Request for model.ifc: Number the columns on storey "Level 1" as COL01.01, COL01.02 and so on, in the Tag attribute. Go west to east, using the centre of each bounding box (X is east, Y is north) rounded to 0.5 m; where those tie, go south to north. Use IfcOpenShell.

First a look at what the model holds.

```python
import ifcopenshell
import ifcopenshell.util.element
import ifcopenshell.util.placement

model = ifcopenshell.open("model.ifc")
print(model.schema)
storey = next(s for s in model.by_type("IfcBuildingStorey") if s.Name == "Level 1")
columns = [e for e in ifcopenshell.util.element.get_decomposition(storey) if e.is_a("IfcColumn")]
for e in sorted(columns, key=lambda e: e.id()):
    origin = ifcopenshell.util.placement.get_local_placement(e.ObjectPlacement)[:3, 3]
    print(e.id(), e.Tag, e.Name, origin.round(2) + 0.0, sep=" | ")
```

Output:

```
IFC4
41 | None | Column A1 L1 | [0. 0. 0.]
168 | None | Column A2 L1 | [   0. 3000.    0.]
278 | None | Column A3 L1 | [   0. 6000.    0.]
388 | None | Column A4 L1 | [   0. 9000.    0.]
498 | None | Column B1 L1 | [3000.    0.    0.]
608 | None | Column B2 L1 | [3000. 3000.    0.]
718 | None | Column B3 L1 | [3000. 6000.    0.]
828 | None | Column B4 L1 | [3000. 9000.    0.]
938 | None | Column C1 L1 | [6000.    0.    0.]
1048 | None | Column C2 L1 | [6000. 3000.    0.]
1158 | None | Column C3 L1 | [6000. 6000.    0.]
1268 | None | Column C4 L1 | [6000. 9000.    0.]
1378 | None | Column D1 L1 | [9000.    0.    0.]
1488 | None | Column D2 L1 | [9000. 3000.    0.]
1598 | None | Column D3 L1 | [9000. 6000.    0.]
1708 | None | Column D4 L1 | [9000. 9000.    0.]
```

```python
import ifcopenshell
import ifcopenshell.geom
import ifcopenshell.util.element
import ifcopenshell.util.shape

model = ifcopenshell.open("model.ifc")
settings = ifcopenshell.geom.settings()
settings.set("use-world-coords", True)


def centre(element):
    shape = ifcopenshell.geom.create_shape(settings, element)
    return ifcopenshell.util.shape.get_bbox_centroid(shape.geometry)


storey = next(s for s in model.by_type("IfcBuildingStorey") if s.Name == "Level 1")
columns = [e for e in ifcopenshell.util.element.get_decomposition(storey) if e.is_a("IfcColumn")]

# Insertion points can sit at a corner or the storey origin, so sort by the geometry (in metres).
centres = {e: centre(e) for e in columns}
columns.sort(key=lambda e: (round(centres[e][0] / 0.5), centres[e][1]))

for i, e in enumerate(columns, start=1):
    number = f"COL01.{i:02d}"
    e.Tag = number
    print(e.id(), number)

model.write("model_rev.ifc")
```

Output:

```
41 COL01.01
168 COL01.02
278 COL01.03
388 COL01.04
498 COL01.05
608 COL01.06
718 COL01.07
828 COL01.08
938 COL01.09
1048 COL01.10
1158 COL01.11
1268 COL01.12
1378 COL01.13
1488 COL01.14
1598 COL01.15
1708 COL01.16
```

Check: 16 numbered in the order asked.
